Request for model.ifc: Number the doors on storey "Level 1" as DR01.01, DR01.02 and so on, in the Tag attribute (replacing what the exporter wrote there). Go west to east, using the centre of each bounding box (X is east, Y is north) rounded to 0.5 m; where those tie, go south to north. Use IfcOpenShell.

First a look at what the model holds.

```python
import ifcopenshell
import ifcopenshell.util.element
import ifcopenshell.util.placement

model = ifcopenshell.open("model.ifc")
print(model.schema)
storey = next(s for s in model.by_type("IfcBuildingStorey") if s.Name == "Level 1")
doors = [e for e in ifcopenshell.util.element.get_decomposition(storey) if e.is_a("IfcDoor")]
for e in sorted(doors, key=lambda e: e.id()):
    origin = ifcopenshell.util.placement.get_local_placement(e.ObjectPlacement)[:3, 3]
    print(e.id(), e.Tag, e.Name, origin.round(2) + 0.0, sep=" | ")
```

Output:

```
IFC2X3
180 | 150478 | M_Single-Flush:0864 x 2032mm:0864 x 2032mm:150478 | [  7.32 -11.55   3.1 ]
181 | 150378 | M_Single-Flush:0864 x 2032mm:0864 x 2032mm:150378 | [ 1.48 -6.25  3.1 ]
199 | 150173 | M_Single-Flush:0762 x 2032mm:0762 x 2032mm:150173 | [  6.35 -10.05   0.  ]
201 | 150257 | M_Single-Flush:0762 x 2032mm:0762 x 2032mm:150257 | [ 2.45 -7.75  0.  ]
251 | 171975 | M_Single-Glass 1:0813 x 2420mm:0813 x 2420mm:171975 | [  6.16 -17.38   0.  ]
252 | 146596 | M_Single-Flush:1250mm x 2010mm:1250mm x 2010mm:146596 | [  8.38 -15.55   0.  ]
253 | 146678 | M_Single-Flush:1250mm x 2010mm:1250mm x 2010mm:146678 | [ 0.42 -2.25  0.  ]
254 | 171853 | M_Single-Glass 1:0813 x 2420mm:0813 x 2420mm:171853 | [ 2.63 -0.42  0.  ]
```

```python
import ifcopenshell
import ifcopenshell.geom
import ifcopenshell.util.element
import ifcopenshell.util.shape

model = ifcopenshell.open("model.ifc")
settings = ifcopenshell.geom.settings()
settings.set("use-world-coords", True)


def centre(element):
    shape = ifcopenshell.geom.create_shape(settings, element)
    return ifcopenshell.util.shape.get_bbox_centroid(shape.geometry)


storey = next(s for s in model.by_type("IfcBuildingStorey") if s.Name == "Level 1")
doors = [e for e in ifcopenshell.util.element.get_decomposition(storey) if e.is_a("IfcDoor")]

# Insertion points can sit at a corner or the storey origin, so sort by the geometry (in metres).
centres = {e: centre(e) for e in doors}
doors.sort(key=lambda e: (round(centres[e][0] / 0.5), centres[e][1]))

for i, e in enumerate(doors, start=1):
    number = f"DR01.{i:02d}"
    e.Tag = number
    print(e.id(), number)

model.write("model_v2.ifc")
```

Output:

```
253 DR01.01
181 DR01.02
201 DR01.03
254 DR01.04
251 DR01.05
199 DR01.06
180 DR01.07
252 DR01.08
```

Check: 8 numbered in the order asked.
